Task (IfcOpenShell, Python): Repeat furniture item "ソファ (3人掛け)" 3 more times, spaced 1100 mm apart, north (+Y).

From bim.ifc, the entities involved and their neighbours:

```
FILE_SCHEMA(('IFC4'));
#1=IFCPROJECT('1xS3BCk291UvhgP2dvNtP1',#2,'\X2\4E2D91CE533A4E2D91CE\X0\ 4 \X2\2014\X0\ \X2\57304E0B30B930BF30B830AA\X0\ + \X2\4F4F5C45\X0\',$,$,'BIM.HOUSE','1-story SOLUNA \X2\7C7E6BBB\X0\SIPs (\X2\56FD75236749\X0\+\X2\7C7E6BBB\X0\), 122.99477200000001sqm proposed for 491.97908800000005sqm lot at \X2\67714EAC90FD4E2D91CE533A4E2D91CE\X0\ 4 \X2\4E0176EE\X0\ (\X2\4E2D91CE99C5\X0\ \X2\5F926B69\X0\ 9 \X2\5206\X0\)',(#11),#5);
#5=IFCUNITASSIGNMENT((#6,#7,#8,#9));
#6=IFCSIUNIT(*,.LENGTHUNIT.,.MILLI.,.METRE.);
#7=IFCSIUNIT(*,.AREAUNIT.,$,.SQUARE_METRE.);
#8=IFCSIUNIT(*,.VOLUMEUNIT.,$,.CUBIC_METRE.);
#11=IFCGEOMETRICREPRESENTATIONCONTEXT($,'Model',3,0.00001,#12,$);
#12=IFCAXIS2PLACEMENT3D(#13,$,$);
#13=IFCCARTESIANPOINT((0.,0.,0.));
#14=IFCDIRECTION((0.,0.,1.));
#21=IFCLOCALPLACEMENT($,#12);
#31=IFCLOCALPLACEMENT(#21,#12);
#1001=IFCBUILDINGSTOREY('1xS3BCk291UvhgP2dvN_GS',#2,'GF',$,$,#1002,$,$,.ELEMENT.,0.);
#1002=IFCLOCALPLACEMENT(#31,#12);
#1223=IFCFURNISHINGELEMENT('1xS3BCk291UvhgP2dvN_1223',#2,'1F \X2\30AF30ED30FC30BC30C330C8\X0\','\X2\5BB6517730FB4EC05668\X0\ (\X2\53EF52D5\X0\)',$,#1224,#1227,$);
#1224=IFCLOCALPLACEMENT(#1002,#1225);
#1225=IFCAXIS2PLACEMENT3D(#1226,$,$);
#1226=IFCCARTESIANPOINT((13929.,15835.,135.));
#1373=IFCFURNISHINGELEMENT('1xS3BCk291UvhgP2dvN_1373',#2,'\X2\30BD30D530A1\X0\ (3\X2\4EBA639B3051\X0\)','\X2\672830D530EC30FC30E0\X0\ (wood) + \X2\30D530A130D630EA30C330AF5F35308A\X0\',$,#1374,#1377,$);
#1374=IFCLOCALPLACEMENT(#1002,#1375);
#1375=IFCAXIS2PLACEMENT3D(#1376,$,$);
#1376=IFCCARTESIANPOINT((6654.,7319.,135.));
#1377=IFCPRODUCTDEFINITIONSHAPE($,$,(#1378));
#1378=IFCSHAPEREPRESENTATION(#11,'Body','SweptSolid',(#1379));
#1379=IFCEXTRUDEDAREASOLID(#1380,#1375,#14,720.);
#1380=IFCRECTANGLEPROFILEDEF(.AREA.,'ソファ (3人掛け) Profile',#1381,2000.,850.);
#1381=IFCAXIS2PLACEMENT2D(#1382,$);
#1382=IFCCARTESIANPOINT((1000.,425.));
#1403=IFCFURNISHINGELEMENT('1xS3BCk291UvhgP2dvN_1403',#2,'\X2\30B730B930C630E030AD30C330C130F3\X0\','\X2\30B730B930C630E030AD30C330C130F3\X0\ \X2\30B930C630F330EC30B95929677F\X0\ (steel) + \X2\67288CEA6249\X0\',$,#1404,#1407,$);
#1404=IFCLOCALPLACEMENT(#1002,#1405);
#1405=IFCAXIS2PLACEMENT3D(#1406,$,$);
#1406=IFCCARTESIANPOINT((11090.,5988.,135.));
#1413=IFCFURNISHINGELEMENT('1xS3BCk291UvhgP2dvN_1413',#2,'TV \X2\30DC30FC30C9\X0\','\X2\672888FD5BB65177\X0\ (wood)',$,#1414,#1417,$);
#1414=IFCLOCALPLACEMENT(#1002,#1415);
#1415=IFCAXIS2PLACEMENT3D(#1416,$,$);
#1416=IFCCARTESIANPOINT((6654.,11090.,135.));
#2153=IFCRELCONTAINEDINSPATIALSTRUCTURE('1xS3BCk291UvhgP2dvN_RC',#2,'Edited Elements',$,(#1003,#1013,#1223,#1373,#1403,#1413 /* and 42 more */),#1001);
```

```python
import numpy as np
import ifcopenshell
import ifcopenshell.api.geometry
import ifcopenshell.api.root
import ifcopenshell.util.element
import ifcopenshell.util.placement
import ifcopenshell.util.unit

model = ifcopenshell.open("bim.ifc")
unit_scale = ifcopenshell.util.unit.calculate_unit_scale(model)


def reuse_history(source, copy):
    """copy_class also copies each property set's owner history, people and application; keep the originals."""
    for rel in copy.IsDefinedBy:
        if rel.is_a("IfcRelDefinesByProperties") and (history := rel.RelatingPropertyDefinition.OwnerHistory):
            rel.RelatingPropertyDefinition.OwnerHistory = source.OwnerHistory
            ifcopenshell.util.element.remove_deep2(model, history)


source = model.by_guid("1xS3BCk291UvhgP2dvN_1373")
base = ifcopenshell.util.placement.get_local_placement(source.ObjectPlacement)
step = np.array([0.0, 1.0, 0.0]) * 1.1 / unit_scale

for i in range(1, 4):
    copy = ifcopenshell.api.root.copy_class(model, product=source)
    copy.Representation = ifcopenshell.util.element.copy_deep(
        model, source.Representation, exclude=["IfcGeometricRepresentationContext", "IfcRepresentationMap"]
    )
    reuse_history(source, copy)
    matrix = base.copy()
    matrix[:3, 3] += i * step
    print("added at", matrix[:3, 3].round(3) + 0.0)
    ifcopenshell.api.geometry.edit_object_placement(model, product=copy, matrix=matrix, is_si=False)

model.write("bim_rev.ifc")
```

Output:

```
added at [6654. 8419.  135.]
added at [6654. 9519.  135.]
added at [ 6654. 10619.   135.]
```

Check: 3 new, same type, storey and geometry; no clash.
